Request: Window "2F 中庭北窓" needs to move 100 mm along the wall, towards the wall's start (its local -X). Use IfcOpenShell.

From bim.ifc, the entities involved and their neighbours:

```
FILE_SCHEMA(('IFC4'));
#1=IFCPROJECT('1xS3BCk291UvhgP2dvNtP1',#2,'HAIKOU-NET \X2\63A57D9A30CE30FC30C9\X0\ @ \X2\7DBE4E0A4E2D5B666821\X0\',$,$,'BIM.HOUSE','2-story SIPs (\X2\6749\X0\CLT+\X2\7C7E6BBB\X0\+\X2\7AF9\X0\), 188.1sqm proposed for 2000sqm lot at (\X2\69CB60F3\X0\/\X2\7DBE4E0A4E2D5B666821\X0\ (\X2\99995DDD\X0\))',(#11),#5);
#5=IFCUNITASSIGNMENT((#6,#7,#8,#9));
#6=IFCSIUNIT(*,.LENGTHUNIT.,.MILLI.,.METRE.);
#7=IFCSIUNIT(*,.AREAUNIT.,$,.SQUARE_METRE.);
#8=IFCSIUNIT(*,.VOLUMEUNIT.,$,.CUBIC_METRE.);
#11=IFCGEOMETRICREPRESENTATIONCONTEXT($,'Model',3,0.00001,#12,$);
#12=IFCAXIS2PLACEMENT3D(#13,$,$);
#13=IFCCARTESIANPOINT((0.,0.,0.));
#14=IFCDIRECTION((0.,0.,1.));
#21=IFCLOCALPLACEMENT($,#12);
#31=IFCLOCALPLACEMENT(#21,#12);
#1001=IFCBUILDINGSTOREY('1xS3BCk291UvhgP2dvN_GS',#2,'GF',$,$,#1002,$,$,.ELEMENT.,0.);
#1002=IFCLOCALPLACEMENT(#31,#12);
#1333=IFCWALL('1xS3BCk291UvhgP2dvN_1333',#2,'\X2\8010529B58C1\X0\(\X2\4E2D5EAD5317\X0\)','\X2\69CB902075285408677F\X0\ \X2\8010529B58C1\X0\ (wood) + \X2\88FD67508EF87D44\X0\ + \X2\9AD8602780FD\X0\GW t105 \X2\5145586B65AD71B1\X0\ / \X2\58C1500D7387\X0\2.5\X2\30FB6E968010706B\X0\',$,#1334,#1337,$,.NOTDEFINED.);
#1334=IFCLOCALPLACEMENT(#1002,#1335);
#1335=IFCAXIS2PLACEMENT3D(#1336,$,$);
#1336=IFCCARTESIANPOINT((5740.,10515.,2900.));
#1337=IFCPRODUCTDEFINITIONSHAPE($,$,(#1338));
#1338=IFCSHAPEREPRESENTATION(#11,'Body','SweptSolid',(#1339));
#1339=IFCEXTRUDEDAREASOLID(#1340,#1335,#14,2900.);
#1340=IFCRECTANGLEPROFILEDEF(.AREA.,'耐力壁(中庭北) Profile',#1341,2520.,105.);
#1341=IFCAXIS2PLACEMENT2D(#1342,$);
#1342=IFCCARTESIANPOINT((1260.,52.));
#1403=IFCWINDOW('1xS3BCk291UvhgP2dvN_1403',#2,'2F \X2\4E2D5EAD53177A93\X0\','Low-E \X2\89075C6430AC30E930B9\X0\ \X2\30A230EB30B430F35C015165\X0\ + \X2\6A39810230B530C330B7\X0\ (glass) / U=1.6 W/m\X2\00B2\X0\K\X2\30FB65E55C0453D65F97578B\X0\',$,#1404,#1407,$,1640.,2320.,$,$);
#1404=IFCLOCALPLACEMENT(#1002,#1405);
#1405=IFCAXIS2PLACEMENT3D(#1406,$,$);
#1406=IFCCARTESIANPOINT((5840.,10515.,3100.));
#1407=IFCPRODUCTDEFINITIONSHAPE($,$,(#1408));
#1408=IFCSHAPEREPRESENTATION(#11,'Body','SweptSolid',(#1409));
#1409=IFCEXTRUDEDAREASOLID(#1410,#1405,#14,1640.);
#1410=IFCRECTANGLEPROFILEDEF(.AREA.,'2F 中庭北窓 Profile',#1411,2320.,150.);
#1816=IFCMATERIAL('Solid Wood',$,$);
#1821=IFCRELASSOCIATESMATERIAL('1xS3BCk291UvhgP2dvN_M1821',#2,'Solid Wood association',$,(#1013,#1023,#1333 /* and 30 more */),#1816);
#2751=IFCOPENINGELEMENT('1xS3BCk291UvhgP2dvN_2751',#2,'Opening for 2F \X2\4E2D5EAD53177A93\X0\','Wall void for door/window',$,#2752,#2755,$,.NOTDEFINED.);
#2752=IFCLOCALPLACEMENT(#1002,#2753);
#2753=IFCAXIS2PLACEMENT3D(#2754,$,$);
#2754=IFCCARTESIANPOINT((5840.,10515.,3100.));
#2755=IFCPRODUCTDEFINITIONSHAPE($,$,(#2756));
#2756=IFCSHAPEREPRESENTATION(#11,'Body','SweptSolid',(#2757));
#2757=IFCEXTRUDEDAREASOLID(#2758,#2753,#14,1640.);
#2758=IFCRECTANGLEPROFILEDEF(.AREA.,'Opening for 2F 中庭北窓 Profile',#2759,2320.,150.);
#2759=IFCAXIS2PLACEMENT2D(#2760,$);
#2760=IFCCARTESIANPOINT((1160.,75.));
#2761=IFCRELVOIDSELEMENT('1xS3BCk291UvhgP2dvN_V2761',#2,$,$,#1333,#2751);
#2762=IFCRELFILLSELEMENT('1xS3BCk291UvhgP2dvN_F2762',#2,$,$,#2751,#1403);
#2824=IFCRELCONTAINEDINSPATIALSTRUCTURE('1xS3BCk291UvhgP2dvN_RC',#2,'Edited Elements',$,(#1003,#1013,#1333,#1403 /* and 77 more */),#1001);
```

```python
import ifcopenshell
import ifcopenshell.api.geometry
import ifcopenshell.util.placement
import ifcopenshell.util.unit

model = ifcopenshell.open("bim.ifc")
unit_scale = ifcopenshell.util.unit.calculate_unit_scale(model)

window = model.by_id(1403)
opening = window.FillsVoids[0].RelatingOpeningElement
wall = opening.VoidsElements[0].RelatingBuildingElement

wall_matrix = ifcopenshell.util.placement.get_local_placement(wall.ObjectPlacement)
shift = wall_matrix[:3, 0] * -0.1 / unit_scale
before = ifcopenshell.util.placement.get_local_placement(window.ObjectPlacement)[:3, 3].copy()

# The window is not placed relative to its opening, so move both.
for product in (opening, window):
    matrix = ifcopenshell.util.placement.get_local_placement(product.ObjectPlacement)
    matrix[:3, 3] += shift
    ifcopenshell.api.geometry.edit_object_placement(model, product=product, matrix=matrix, is_si=False)

after = ifcopenshell.util.placement.get_local_placement(window.ObjectPlacement)[:3, 3]
print("window moved by", (after - before).round(3) + 0.0)

model.write("bim_v2.ifc")
```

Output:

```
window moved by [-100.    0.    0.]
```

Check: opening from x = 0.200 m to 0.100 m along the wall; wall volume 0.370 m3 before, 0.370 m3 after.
